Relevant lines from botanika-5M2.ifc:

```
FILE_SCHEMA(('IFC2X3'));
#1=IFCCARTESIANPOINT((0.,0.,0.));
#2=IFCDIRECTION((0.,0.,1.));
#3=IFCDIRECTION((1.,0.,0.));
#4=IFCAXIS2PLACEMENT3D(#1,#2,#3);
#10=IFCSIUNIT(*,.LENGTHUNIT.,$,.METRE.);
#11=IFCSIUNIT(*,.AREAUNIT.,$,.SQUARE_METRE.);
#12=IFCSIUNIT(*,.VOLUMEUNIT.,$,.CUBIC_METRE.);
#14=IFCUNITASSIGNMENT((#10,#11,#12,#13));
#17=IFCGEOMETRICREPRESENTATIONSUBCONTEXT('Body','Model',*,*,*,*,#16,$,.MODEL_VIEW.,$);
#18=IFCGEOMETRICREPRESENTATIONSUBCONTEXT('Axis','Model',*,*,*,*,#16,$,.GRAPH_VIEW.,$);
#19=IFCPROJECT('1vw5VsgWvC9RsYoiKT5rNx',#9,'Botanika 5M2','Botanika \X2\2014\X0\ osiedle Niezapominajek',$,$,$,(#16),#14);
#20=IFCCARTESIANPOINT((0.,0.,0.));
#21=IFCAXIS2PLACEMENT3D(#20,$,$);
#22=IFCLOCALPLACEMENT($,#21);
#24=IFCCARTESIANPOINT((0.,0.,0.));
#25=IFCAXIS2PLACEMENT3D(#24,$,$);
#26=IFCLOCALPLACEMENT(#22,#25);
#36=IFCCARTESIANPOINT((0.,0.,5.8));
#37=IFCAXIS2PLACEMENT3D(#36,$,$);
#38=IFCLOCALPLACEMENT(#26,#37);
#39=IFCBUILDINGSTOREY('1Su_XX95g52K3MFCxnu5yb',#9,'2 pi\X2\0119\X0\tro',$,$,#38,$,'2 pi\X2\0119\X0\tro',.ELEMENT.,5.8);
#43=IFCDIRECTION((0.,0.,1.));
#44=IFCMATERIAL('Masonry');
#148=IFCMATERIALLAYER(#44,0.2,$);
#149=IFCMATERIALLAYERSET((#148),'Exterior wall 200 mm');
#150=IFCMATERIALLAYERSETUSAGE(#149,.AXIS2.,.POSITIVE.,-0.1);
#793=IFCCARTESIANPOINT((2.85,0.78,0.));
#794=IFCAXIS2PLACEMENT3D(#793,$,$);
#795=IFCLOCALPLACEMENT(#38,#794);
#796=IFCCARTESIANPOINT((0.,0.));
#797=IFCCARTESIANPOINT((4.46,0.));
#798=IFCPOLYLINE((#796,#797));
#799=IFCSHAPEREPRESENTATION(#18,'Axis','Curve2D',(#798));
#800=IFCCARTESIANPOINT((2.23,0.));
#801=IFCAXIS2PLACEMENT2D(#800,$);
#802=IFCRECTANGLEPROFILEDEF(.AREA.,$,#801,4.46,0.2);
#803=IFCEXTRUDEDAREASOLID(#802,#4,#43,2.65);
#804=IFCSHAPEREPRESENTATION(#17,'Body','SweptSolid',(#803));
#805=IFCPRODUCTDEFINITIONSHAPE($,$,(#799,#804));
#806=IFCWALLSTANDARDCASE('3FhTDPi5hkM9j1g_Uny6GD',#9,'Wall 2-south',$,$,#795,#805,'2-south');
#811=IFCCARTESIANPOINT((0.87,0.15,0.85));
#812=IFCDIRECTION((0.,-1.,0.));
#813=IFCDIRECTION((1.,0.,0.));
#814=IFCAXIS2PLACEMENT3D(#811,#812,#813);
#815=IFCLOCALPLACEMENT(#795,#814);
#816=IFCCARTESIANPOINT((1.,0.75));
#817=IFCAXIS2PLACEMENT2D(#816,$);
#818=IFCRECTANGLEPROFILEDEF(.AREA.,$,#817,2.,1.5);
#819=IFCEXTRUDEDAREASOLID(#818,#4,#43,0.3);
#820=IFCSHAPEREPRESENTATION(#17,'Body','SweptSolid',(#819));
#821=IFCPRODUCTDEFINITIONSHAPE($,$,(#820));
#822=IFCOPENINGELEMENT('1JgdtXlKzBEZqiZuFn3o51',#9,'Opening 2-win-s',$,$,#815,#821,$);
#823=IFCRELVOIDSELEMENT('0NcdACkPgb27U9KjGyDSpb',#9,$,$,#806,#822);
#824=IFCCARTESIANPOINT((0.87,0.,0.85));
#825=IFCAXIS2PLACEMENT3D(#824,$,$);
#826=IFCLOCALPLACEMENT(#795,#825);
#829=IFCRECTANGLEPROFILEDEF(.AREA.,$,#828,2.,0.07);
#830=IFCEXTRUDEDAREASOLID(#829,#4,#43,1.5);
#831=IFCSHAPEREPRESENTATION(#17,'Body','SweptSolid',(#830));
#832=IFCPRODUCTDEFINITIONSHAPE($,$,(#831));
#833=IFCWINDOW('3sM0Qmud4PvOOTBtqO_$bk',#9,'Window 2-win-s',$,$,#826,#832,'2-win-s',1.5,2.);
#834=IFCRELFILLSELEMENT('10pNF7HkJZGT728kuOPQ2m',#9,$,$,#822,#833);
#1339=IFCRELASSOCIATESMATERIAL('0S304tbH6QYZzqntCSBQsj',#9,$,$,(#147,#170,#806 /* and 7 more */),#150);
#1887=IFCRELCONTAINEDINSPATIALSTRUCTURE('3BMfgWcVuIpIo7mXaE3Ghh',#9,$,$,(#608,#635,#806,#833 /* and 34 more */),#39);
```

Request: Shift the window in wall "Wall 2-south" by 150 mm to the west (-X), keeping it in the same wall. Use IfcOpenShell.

```python
import ifcopenshell
import ifcopenshell.api.geometry
import ifcopenshell.util.placement
import ifcopenshell.util.unit

model = ifcopenshell.open("botanika-5M2.ifc")
unit_scale = ifcopenshell.util.unit.calculate_unit_scale(model)

window = model.by_guid("3sM0Qmud4PvOOTBtqO_$bk")
opening = window.FillsVoids[0].RelatingOpeningElement
wall = opening.VoidsElements[0].RelatingBuildingElement

wall_matrix = ifcopenshell.util.placement.get_local_placement(wall.ObjectPlacement)
shift = wall_matrix[:3, 0] * -0.15 / unit_scale
before = ifcopenshell.util.placement.get_local_placement(window.ObjectPlacement)[:3, 3].copy()

# The window is not placed relative to its opening, so move both.
for product in (opening, window):
    matrix = ifcopenshell.util.placement.get_local_placement(product.ObjectPlacement)
    matrix[:3, 3] += shift
    ifcopenshell.api.geometry.edit_object_placement(model, product=product, matrix=matrix, is_si=False)

after = ifcopenshell.util.placement.get_local_placement(window.ObjectPlacement)[:3, 3]
print("window moved by", (after - before).round(3) + 0.0)

model.write("botanika-5M2_v2.ifc")
```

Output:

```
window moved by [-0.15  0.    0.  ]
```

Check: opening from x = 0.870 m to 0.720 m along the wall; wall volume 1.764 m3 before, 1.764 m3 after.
